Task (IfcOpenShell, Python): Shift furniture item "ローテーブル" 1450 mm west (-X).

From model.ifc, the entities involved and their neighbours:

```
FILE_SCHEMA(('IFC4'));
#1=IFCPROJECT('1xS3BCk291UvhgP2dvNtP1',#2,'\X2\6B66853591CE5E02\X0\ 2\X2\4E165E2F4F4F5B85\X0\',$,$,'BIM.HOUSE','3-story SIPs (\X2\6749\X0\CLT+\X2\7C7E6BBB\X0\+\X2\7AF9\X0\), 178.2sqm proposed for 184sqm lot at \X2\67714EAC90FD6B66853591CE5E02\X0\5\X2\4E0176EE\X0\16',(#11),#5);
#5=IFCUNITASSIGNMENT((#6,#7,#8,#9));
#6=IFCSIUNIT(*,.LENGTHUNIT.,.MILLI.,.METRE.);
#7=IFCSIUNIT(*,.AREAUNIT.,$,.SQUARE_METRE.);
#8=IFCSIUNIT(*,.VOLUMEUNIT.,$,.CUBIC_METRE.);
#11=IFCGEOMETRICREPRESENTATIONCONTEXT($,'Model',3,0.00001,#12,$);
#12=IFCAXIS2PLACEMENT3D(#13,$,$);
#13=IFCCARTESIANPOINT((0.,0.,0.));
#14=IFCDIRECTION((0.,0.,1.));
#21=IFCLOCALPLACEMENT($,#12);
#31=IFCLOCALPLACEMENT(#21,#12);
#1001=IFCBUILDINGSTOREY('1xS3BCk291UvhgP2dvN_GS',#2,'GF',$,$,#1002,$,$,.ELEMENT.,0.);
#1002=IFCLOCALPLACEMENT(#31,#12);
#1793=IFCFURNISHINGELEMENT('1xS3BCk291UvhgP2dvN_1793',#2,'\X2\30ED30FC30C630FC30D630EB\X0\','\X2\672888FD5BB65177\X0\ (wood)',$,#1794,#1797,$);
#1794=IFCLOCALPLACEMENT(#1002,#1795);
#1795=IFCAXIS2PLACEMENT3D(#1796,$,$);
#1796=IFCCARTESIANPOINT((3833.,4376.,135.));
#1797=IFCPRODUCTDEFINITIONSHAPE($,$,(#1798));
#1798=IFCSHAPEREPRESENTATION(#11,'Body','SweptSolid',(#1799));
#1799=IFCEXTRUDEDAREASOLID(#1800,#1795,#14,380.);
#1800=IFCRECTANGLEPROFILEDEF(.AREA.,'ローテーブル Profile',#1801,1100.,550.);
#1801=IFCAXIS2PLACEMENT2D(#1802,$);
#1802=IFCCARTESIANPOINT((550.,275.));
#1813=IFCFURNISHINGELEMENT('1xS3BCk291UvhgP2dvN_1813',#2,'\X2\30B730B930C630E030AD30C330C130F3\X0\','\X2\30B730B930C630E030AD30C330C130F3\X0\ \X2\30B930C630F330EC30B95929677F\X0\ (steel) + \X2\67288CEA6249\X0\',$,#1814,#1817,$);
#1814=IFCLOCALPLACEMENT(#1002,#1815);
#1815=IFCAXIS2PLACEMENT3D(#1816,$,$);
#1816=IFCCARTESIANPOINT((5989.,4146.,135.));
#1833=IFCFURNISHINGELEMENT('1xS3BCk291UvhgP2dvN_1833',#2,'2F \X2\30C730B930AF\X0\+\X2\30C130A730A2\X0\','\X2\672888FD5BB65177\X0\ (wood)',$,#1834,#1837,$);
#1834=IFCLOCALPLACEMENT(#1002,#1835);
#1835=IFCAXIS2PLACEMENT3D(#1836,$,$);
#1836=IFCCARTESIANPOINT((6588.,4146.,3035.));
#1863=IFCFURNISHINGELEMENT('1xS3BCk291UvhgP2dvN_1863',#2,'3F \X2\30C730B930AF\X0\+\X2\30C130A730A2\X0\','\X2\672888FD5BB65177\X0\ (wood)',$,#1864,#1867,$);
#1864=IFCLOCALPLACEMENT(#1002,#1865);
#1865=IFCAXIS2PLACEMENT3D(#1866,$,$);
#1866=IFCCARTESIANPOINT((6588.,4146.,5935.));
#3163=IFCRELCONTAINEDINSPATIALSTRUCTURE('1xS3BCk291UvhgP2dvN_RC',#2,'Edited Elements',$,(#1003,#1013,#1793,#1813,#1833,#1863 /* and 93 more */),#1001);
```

```python
import ifcopenshell
import ifcopenshell.api.geometry
import ifcopenshell.util.placement
import ifcopenshell.util.unit

model = ifcopenshell.open("model.ifc")
unit_scale = ifcopenshell.util.unit.calculate_unit_scale(model)

item = model.by_guid("1xS3BCk291UvhgP2dvN_1793")
matrix = ifcopenshell.util.placement.get_local_placement(item.ObjectPlacement)
matrix[0, 3] -= 1.45 / unit_scale
ifcopenshell.api.geometry.edit_object_placement(model, product=item, matrix=matrix, is_si=False)

print(ifcopenshell.util.placement.get_local_placement(item.ObjectPlacement).round(3) + 0.0)

model.write("model-out.ifc")
```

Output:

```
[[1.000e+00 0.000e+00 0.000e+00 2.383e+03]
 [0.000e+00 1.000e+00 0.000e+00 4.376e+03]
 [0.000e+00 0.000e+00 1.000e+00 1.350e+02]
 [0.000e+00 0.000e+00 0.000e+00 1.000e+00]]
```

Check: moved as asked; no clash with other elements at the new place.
